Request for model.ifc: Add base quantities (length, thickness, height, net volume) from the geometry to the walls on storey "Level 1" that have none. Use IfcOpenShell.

First a look at what the model holds.

```python
import ifcopenshell
import ifcopenshell.util.element
import ifcopenshell.util.unit

model = ifcopenshell.open("model.ifc")
print(model.schema)
for unit_type in ("LENGTHUNIT", "AREAUNIT", "VOLUMEUNIT"):
    print(unit_type, ifcopenshell.util.unit.calculate_unit_scale(model, unit_type))
storey = next(s for s in model.by_type("IfcBuildingStorey") if s.Name == "Level 1")
walls = [e for e in ifcopenshell.util.element.get_decomposition(storey) if e.is_a("IfcWall")]
for e in sorted(walls, key=lambda e: e.id()):
    print(e.id(), e.is_a(), e.Name, list(ifcopenshell.util.element.get_psets(e, qtos_only=True)), sep=" | ")
```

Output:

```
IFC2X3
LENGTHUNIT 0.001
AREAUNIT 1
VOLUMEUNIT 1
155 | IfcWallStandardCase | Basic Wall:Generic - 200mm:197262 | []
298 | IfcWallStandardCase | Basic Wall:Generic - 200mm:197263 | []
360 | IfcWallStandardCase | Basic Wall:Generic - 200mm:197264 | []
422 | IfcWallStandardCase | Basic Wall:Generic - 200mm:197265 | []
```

```python
import ifcopenshell
import ifcopenshell.api.pset
import ifcopenshell.geom
import ifcopenshell.util.element
import ifcopenshell.util.shape
import ifcopenshell.util.unit

model = ifcopenshell.open("model.ifc")
unit_scale = ifcopenshell.util.unit.calculate_unit_scale(model)
volume_scale = ifcopenshell.util.unit.calculate_unit_scale(model, "VOLUMEUNIT")
settings = ifcopenshell.geom.settings()

storey = next(s for s in model.by_type("IfcBuildingStorey") if s.Name == "Level 1")
walls = [e for e in ifcopenshell.util.element.get_decomposition(storey) if e.is_a("IfcWall")]

for e in sorted(walls, key=lambda e: e.id()):
    if ifcopenshell.util.element.get_psets(e, qtos_only=True, should_inherit=False):
        continue
    # Geometry comes back in metres, in the element's own axes.
    shape = ifcopenshell.geom.create_shape(settings, e)
    values = {
        "Length": ifcopenshell.util.shape.get_x(shape.geometry) / unit_scale,
        "Width": ifcopenshell.util.shape.get_y(shape.geometry) / unit_scale,
        "Height": ifcopenshell.util.shape.get_z(shape.geometry) / unit_scale,
        "NetVolume": ifcopenshell.util.shape.get_volume(shape.geometry) / volume_scale,
    }
    qto = ifcopenshell.api.pset.add_qto(model, product=e, name="BaseQuantities")
    ifcopenshell.api.pset.edit_qto(model, qto=qto, properties=values)
    print(e.id(), {k: round(v, 3) for k, v in values.items()})

model.write("model_edited.ifc")
```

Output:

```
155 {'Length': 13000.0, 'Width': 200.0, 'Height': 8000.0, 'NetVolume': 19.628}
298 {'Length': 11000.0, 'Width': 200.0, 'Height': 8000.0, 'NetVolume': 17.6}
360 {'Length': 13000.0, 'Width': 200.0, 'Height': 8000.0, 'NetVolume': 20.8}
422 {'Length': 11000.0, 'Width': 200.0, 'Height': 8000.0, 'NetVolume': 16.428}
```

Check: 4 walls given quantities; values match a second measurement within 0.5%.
